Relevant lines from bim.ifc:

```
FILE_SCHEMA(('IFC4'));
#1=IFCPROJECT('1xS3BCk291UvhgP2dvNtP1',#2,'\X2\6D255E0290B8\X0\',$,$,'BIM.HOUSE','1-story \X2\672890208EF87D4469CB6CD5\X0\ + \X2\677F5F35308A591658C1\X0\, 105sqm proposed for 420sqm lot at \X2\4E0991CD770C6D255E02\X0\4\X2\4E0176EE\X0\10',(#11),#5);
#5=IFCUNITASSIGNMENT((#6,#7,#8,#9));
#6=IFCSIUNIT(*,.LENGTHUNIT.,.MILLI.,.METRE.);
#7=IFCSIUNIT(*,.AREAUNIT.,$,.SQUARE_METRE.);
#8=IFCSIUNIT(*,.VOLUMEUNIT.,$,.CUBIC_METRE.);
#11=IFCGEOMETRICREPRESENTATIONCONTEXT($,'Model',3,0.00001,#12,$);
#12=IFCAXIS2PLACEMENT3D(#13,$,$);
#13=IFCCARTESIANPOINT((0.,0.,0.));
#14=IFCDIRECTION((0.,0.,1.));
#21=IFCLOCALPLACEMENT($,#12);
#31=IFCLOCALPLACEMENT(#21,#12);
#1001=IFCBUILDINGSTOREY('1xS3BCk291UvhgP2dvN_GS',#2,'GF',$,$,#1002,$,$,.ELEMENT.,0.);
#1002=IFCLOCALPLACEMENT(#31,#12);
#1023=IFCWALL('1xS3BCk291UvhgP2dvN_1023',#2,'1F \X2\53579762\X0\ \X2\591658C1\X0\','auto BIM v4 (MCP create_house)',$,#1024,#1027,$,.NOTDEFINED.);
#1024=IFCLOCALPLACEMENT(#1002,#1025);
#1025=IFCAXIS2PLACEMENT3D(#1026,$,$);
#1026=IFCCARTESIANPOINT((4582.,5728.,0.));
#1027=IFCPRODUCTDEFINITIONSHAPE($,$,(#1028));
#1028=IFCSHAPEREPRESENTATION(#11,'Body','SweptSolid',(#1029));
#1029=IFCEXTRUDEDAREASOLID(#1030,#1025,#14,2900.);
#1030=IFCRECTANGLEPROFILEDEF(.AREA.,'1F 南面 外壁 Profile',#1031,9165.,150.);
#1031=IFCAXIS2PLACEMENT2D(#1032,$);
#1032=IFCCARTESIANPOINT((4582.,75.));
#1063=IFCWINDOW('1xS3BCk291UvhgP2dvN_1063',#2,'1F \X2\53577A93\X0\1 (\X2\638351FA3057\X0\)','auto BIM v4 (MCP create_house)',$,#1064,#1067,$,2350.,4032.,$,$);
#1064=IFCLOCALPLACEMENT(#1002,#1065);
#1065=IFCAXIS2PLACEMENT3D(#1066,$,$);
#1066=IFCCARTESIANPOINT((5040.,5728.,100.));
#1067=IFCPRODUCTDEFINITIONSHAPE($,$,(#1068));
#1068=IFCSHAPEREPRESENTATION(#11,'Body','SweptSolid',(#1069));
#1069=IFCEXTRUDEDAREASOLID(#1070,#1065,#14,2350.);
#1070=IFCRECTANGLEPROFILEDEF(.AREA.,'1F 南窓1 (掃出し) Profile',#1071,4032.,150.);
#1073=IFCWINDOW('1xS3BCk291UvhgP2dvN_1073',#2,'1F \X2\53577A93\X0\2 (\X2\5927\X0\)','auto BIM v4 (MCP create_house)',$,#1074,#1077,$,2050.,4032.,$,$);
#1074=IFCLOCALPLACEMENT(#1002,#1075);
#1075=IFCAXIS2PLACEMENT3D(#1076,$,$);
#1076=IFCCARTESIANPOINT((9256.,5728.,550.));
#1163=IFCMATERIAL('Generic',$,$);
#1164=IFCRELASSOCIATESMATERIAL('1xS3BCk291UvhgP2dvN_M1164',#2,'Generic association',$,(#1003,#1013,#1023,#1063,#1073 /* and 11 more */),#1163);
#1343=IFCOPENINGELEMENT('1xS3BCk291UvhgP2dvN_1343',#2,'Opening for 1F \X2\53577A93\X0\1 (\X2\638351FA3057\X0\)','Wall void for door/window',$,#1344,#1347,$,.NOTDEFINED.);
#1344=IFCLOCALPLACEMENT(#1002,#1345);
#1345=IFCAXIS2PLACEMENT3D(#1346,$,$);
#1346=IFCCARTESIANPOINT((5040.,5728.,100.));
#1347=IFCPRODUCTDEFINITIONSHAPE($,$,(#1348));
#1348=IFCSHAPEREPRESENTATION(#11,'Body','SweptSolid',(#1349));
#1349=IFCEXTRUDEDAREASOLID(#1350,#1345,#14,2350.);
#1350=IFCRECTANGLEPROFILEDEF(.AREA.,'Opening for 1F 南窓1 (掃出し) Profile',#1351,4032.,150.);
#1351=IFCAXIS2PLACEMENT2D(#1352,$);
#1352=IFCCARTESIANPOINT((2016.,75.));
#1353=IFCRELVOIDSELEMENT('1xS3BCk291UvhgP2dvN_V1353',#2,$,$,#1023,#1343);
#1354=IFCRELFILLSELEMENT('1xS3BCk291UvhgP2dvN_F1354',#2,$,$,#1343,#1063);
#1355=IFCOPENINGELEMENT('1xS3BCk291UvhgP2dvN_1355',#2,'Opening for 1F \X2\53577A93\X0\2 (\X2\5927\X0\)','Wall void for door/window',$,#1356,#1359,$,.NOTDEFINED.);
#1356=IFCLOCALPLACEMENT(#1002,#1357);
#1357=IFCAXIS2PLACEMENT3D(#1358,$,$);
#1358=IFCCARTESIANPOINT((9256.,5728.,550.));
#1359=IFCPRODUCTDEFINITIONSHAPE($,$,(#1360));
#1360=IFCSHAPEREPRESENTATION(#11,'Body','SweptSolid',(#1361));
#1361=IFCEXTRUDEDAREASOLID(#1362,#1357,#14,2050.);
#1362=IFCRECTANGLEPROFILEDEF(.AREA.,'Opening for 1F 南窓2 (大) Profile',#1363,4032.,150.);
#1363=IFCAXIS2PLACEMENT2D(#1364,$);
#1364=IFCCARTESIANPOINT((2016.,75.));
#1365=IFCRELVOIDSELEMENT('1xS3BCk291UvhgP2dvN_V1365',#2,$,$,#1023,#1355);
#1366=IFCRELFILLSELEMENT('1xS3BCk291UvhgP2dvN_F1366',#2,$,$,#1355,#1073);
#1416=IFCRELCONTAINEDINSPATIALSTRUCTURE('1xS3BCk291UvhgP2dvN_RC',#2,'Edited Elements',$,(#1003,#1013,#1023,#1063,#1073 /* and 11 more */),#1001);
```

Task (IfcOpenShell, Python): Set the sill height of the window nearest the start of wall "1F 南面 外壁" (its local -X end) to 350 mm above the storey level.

```python
import numpy as np
import ifcopenshell
import ifcopenshell.api.geometry
import ifcopenshell.geom
import ifcopenshell.util.element
import ifcopenshell.util.placement
import ifcopenshell.util.shape
import ifcopenshell.util.unit

model = ifcopenshell.open("bim.ifc")
unit_scale = ifcopenshell.util.unit.calculate_unit_scale(model)

window = model.by_guid("1xS3BCk291UvhgP2dvN_1063")
opening = window.FillsVoids[0].RelatingOpeningElement
storey = ifcopenshell.util.element.get_container(window, ifc_class="IfcBuildingStorey")
level = ifcopenshell.util.placement.get_local_placement(storey.ObjectPlacement)[2, 3]

# The opening's origin need not be at the sill, so measure its lowest point.
shape = ifcopenshell.geom.create_shape(ifcopenshell.geom.settings(), opening)
bottom = ifcopenshell.util.shape.get_shape_bottom_elevation(shape, shape.geometry) / unit_scale
dz = level + 0.35 / unit_scale - bottom

shift = np.array([0.0, 0.0, dz])
# The window is not placed relative to its opening, so move both.
for product in (opening, window):
    matrix = ifcopenshell.util.placement.get_local_placement(product.ObjectPlacement)
    matrix[:3, 3] += shift
    ifcopenshell.api.geometry.edit_object_placement(model, product=product, matrix=matrix, is_si=False)

print(f"moved by {dz * unit_scale:+.3f} m")

model.write("bim_rev.ifc")
```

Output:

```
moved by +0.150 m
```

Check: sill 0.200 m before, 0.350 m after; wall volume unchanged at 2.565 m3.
